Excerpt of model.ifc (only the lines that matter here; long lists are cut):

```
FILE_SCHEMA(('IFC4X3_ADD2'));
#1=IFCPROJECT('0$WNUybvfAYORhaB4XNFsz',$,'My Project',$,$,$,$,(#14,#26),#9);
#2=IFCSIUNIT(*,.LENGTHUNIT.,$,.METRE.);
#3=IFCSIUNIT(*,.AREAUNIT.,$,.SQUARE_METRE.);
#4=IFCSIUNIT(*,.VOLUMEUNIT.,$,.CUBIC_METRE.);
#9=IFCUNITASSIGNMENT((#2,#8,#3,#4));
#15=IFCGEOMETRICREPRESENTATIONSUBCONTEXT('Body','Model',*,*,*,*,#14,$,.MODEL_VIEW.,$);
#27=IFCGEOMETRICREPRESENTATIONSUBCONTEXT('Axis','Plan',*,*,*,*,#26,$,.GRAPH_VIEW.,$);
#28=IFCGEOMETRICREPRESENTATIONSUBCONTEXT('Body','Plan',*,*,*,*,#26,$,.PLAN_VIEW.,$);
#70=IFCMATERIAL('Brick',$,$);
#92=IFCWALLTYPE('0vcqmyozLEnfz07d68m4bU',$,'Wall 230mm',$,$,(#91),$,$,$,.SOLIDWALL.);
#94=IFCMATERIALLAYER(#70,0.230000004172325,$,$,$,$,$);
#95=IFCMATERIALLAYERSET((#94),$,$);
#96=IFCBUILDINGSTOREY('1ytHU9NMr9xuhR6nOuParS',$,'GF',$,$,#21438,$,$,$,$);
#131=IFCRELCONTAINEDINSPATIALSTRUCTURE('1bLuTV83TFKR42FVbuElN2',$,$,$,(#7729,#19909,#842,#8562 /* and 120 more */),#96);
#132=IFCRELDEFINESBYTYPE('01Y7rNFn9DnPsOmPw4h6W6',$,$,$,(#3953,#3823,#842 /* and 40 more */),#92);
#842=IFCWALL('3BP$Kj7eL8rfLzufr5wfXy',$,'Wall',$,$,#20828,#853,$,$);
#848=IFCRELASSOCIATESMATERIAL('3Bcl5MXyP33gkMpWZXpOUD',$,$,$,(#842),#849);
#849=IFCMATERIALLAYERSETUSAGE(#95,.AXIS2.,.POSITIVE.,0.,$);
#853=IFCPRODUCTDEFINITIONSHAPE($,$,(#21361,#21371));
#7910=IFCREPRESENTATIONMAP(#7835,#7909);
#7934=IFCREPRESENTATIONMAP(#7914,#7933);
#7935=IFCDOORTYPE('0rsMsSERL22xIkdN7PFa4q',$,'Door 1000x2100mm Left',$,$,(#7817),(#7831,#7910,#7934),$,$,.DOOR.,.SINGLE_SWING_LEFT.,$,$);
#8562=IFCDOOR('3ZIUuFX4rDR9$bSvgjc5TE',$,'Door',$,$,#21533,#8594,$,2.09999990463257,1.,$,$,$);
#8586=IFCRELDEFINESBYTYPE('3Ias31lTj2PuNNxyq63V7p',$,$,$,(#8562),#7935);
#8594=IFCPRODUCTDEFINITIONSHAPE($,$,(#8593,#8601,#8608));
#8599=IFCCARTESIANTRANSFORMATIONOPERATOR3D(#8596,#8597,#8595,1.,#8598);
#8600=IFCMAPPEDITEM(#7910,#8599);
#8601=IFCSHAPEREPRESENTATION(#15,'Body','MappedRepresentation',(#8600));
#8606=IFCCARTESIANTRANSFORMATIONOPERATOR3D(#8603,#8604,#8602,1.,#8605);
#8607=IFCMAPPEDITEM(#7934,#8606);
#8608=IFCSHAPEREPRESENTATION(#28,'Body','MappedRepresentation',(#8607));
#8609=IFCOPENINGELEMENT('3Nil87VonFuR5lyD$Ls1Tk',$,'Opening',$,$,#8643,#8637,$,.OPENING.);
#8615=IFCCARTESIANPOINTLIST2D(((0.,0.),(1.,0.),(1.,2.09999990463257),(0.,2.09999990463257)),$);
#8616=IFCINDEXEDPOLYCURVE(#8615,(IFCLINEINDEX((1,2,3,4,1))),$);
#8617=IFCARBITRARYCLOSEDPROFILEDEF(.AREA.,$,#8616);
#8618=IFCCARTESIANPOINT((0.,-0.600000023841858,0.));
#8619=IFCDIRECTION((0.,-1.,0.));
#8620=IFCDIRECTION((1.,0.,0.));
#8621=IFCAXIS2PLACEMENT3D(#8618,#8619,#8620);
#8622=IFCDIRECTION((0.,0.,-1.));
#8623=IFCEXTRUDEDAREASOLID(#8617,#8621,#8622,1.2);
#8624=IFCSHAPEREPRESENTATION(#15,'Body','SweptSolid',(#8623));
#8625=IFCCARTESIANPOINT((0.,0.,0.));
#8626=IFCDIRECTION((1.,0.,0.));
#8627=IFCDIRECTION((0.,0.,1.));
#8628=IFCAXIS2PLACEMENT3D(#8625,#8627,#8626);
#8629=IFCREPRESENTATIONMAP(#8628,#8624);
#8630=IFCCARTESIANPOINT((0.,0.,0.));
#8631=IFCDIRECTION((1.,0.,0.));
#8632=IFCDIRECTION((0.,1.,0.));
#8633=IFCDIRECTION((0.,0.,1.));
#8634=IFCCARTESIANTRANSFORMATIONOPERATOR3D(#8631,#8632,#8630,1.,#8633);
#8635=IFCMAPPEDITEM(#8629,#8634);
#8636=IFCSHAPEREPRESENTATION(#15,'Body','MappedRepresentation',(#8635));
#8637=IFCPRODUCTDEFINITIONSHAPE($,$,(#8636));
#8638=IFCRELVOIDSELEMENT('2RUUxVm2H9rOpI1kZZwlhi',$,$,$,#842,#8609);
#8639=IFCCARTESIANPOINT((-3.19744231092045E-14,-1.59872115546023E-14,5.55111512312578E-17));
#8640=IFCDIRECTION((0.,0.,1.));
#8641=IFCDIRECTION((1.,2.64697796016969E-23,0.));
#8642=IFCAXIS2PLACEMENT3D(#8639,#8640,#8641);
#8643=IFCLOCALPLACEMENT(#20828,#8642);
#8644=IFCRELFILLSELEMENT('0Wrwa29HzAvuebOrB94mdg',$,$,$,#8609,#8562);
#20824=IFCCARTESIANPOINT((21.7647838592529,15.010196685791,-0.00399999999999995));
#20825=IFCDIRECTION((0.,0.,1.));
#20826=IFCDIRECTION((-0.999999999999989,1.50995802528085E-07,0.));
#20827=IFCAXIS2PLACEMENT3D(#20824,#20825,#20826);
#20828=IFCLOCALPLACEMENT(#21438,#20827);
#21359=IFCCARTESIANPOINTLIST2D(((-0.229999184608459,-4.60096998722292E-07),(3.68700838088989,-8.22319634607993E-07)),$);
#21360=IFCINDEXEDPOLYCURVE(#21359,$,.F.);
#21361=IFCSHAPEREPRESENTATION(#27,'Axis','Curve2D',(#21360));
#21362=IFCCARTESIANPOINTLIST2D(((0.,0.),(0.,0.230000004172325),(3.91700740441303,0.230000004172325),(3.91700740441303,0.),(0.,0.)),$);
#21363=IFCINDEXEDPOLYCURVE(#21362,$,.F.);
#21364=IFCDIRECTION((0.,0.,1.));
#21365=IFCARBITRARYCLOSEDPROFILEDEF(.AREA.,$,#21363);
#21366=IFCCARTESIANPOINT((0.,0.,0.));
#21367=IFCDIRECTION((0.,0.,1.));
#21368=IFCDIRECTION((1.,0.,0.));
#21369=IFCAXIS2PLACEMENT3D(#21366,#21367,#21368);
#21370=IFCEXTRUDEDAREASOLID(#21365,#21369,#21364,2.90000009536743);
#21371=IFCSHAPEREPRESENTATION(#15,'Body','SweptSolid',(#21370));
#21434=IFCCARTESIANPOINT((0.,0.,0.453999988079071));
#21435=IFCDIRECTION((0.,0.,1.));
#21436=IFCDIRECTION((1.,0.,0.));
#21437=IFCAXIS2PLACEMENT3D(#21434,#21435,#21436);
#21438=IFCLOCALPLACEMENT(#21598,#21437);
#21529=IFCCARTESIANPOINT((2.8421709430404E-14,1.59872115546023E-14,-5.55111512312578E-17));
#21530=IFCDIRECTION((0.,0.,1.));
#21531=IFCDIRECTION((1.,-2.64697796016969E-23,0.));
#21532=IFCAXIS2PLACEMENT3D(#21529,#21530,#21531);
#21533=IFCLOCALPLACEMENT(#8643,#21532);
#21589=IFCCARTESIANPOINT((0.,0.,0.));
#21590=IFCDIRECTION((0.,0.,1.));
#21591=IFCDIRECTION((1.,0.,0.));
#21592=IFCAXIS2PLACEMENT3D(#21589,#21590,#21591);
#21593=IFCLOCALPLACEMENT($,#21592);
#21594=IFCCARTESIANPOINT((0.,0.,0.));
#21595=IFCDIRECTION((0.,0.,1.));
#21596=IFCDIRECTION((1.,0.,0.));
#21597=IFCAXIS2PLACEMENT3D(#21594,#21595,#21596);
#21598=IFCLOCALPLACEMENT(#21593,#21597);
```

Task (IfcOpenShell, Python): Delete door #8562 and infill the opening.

```python
import ifcopenshell
import ifcopenshell.api.feature
import ifcopenshell.api.root
import ifcopenshell.geom
import ifcopenshell.util.shape

model = ifcopenshell.open("model.ifc")
settings = ifcopenshell.geom.settings()


def volume(element):
    """Net volume in cubic metres, openings subtracted."""
    shape = ifcopenshell.geom.create_shape(settings, element)
    return ifcopenshell.util.shape.get_volume(shape.geometry)


door = model.by_id(8562)
opening = door.FillsVoids[0].RelatingOpeningElement
wall = opening.VoidsElements[0].RelatingBuildingElement
before = volume(wall)

ifcopenshell.api.root.remove_product(model, product=door)
ifcopenshell.api.feature.remove_feature(model, feature=opening)

after = volume(wall)

print(f"wall volume {before:.3f} -> {after:.3f} m3")

model.write("model-out.ifc")
```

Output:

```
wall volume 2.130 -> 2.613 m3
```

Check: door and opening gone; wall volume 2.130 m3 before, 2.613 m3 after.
